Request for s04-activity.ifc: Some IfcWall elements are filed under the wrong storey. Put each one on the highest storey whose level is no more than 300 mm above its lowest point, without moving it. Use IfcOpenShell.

First a look at what the model holds.

```python
import ifcopenshell
import ifcopenshell.util.element
import ifcopenshell.util.placement

model = ifcopenshell.open("s04-activity.ifc")
print(model.schema)
for storey in model.by_type("IfcBuildingStorey"):
    level = ifcopenshell.util.placement.get_storey_elevation(storey)
    count = sum(e.is_a("IfcWall") for e in ifcopenshell.util.element.get_contained(storey))
    print(storey.id(), storey.Name, round(level, 3), count, sep=" | ")
```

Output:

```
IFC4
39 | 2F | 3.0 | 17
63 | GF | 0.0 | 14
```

```python
import ifcopenshell
import ifcopenshell.api.spatial
import ifcopenshell.geom
import ifcopenshell.util.element
import ifcopenshell.util.placement
import ifcopenshell.util.shape
import ifcopenshell.util.unit

model = ifcopenshell.open("s04-activity.ifc")
unit_scale = ifcopenshell.util.unit.calculate_unit_scale(model)
settings = ifcopenshell.geom.settings()

levels = sorted(
    ((ifcopenshell.util.placement.get_storey_elevation(s) * unit_scale, s) for s in model.by_type("IfcBuildingStorey")),
    key=lambda pair: pair[0],
)

for e in model.by_type("IfcWall"):
    current = e.ContainedInStructure[0].RelatingStructure if e.ContainedInStructure else None
    if current is None or not current.is_a("IfcBuildingStorey"):
        continue
    shape = ifcopenshell.geom.create_shape(settings, e)
    bottom = ifcopenshell.util.shape.get_shape_bottom_elevation(shape, shape.geometry)
    below = [s for level, s in levels if level <= bottom + 0.3]
    storey = below[-1] if below else levels[0][1]
    if storey != current:
        # assign_container keeps the world position.
        ifcopenshell.api.spatial.assign_container(model, products=[e], relating_structure=storey)
        print(e.id(), current.Name, "->", storey.Name)

model.write("s04-activity_v2.ifc")
```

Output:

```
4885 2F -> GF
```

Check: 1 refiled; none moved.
